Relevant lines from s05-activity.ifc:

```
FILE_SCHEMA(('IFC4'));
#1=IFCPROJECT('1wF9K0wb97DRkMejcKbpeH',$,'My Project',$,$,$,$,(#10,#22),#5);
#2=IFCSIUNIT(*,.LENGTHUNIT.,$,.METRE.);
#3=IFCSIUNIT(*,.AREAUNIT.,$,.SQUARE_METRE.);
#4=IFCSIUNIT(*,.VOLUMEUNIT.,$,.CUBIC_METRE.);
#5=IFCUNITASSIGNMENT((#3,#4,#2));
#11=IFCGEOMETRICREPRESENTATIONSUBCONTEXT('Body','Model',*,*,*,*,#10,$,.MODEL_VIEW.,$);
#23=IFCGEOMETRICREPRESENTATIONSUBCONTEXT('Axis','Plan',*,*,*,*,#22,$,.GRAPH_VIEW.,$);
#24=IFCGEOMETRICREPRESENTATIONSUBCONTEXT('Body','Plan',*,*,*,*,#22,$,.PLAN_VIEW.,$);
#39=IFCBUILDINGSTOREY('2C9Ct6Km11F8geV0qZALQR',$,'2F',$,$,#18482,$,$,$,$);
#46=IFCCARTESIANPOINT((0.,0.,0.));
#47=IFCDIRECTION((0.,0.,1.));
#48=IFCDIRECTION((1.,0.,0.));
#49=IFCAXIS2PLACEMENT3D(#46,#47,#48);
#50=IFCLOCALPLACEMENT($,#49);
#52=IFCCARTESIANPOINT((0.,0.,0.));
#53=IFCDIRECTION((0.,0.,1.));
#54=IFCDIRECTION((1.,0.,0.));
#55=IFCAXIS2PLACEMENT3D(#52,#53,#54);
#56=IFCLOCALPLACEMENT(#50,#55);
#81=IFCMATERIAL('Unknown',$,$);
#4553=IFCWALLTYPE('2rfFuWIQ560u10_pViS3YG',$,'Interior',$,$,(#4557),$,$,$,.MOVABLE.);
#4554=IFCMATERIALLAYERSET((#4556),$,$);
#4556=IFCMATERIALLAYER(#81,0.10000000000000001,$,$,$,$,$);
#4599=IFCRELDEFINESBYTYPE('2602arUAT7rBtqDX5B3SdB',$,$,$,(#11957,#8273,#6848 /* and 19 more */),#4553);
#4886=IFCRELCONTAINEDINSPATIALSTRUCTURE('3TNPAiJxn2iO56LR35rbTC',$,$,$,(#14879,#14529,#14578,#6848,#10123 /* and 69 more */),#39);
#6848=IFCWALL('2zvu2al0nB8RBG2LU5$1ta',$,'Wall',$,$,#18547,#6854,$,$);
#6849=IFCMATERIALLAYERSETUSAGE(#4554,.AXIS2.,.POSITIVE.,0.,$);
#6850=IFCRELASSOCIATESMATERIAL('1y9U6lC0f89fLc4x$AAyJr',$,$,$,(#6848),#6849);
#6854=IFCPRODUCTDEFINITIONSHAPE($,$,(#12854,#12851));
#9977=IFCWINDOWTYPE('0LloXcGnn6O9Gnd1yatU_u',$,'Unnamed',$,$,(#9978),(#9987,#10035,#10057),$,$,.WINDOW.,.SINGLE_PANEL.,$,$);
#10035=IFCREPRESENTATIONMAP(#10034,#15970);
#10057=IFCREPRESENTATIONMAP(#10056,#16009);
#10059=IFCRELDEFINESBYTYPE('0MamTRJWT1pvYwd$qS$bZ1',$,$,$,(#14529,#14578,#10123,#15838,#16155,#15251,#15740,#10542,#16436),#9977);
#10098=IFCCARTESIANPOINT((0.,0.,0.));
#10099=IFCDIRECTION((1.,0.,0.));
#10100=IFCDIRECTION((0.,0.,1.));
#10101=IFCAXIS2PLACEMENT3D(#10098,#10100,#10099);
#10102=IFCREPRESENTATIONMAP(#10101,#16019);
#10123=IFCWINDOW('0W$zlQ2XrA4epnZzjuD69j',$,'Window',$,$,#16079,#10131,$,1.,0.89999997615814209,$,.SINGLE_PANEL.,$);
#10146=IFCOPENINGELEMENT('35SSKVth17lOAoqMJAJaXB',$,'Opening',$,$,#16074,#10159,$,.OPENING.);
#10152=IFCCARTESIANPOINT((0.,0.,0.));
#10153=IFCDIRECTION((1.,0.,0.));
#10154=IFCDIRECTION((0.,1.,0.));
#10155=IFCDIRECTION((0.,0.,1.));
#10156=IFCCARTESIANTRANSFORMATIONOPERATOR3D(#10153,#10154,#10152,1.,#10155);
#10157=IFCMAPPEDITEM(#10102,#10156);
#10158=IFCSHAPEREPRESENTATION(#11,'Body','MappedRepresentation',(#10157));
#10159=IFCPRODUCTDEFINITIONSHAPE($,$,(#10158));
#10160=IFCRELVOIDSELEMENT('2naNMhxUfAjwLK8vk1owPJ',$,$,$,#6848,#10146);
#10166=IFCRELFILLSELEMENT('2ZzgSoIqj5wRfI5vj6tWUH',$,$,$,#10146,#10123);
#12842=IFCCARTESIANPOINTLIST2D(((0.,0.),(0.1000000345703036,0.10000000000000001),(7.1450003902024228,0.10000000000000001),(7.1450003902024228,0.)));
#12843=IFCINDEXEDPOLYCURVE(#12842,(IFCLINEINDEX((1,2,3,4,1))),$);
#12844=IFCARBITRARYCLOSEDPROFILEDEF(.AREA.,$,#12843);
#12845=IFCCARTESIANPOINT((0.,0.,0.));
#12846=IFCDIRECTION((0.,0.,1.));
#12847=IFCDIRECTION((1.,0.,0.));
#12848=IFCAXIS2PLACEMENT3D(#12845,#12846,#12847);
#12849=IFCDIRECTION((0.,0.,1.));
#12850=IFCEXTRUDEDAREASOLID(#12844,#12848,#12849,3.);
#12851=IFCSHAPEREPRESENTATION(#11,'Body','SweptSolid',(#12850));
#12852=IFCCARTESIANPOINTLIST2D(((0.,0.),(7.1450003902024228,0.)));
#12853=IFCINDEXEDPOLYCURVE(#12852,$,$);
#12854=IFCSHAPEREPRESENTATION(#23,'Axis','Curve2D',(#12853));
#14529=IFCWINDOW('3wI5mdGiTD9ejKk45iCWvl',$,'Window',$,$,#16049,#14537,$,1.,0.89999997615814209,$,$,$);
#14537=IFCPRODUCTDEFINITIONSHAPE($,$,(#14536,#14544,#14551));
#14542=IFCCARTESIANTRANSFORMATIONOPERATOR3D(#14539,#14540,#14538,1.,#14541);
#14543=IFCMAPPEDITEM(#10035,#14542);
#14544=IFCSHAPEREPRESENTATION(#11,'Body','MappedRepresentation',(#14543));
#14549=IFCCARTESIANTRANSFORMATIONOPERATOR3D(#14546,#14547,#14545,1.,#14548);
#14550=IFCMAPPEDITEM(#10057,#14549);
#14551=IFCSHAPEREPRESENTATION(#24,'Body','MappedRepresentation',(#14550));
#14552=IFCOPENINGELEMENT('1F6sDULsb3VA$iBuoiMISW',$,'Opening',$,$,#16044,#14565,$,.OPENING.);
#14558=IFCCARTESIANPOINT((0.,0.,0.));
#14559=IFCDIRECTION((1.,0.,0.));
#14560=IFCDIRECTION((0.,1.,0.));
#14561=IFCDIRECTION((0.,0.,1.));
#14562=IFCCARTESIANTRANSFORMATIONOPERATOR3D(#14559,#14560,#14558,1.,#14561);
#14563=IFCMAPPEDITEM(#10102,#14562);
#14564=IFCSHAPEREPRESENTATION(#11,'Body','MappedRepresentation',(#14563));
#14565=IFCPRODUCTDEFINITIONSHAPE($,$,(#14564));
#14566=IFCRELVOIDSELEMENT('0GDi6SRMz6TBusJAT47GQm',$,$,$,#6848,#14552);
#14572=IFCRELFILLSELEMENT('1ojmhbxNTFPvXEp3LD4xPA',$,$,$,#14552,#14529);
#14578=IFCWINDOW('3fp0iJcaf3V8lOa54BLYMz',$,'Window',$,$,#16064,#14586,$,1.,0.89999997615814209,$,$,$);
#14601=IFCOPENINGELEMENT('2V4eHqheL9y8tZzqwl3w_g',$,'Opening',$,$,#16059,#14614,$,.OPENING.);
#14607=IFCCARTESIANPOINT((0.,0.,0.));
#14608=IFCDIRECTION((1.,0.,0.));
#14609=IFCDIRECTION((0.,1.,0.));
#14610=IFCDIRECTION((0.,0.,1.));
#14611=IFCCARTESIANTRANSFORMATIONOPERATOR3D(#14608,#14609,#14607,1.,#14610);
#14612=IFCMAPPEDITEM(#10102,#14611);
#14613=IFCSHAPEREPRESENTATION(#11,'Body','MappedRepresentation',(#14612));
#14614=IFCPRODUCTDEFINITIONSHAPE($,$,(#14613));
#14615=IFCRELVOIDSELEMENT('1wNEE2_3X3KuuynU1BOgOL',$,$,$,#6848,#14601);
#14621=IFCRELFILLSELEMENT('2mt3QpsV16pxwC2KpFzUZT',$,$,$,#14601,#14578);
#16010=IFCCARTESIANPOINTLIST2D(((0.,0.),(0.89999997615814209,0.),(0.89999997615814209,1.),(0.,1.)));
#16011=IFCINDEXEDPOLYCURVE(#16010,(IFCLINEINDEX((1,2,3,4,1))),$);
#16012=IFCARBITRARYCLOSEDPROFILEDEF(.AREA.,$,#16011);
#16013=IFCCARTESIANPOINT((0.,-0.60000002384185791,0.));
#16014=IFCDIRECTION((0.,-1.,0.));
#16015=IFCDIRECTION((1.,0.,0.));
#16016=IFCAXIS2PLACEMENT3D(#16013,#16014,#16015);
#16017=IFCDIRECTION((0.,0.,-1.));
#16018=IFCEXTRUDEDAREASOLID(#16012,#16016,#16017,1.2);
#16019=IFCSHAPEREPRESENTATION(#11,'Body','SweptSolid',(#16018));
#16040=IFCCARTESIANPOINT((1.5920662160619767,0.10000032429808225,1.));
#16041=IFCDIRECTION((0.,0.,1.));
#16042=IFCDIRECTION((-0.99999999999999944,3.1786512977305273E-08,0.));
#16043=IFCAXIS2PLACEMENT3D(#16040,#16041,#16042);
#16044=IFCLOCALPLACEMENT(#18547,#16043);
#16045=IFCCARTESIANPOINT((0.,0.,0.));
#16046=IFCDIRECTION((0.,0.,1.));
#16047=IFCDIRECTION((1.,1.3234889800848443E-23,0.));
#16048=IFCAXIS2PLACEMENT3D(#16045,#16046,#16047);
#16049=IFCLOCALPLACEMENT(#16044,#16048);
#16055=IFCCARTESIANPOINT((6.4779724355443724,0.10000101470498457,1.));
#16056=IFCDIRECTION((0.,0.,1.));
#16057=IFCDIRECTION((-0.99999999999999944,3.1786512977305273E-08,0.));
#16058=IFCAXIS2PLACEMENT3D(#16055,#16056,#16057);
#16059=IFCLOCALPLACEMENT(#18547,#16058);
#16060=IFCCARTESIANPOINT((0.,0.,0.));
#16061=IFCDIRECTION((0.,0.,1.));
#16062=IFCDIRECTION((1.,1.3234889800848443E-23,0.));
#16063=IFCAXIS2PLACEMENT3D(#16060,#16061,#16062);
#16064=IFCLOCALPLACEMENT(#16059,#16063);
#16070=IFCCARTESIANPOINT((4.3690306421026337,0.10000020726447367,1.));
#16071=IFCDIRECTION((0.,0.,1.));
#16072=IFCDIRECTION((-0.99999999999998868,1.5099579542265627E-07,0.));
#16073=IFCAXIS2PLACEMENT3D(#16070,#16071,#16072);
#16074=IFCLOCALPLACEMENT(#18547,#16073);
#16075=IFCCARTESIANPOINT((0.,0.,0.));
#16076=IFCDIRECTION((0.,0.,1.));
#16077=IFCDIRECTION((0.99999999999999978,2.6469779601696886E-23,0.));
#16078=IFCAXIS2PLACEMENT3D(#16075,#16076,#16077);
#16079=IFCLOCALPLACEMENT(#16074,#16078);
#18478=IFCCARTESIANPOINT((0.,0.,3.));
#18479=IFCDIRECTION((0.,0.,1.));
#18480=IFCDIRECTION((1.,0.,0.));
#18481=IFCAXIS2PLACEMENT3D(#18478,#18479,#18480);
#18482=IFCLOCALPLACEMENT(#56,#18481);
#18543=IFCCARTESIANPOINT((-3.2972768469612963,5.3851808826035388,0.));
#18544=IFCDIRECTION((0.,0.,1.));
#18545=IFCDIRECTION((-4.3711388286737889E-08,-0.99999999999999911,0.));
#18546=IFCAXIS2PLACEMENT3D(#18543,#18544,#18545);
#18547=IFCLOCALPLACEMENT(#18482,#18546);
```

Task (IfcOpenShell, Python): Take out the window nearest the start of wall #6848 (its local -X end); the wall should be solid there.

```python
import ifcopenshell
import ifcopenshell.api.feature
import ifcopenshell.api.root
import ifcopenshell.geom
import ifcopenshell.util.shape

model = ifcopenshell.open("s05-activity.ifc")
settings = ifcopenshell.geom.settings()


def volume(element):
    """Net volume in cubic metres, openings subtracted."""
    shape = ifcopenshell.geom.create_shape(settings, element)
    return ifcopenshell.util.shape.get_volume(shape.geometry)


window = model.by_guid("3wI5mdGiTD9ejKk45iCWvl")
opening = window.FillsVoids[0].RelatingOpeningElement
wall = opening.VoidsElements[0].RelatingBuildingElement
before = volume(wall)

ifcopenshell.api.root.remove_product(model, product=window)
ifcopenshell.api.feature.remove_feature(model, feature=opening)

after = volume(wall)

print(f"wall volume {before:.3f} -> {after:.3f} m3")

model.write("s05-activity_rev.ifc")
```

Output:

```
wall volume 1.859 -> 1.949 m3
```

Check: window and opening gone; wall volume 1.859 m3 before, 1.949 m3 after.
